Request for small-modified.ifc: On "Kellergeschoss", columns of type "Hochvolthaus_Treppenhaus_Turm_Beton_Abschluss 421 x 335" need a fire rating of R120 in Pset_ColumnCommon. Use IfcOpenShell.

First a look at what the model holds.

```python
import ifcopenshell
import ifcopenshell.util.element

model = ifcopenshell.open("small-modified.ifc")
print(model.schema)
storey = next(s for s in model.by_type("IfcBuildingStorey") if s.Name == "Kellergeschoss")
columns = [e for e in ifcopenshell.util.element.get_decomposition(storey) if e.is_a("IfcColumn")]
seen = {}
for e in columns:
    element_type = ifcopenshell.util.element.get_type(e)
    key = (element_type.Name if element_type != e and element_type else None, ifcopenshell.util.element.get_pset(e, "Pset_ColumnCommon", "FireRating"))
    seen[key] = seen.get(key, 0) + 1
for (name, value), count in sorted(seen.items(), key=str):
    print(count, "x", name, "|", value)
```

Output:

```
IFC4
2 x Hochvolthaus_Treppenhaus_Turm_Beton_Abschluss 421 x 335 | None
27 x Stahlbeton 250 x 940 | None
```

```python
import ifcopenshell
import ifcopenshell.api.pset
import ifcopenshell.util.element

model = ifcopenshell.open("small-modified.ifc")

storey = next(s for s in model.by_type("IfcBuildingStorey") if s.Name == "Kellergeschoss")
columns = [e for e in ifcopenshell.util.element.get_decomposition(storey) if e.is_a("IfcColumn")]

count = 0
for e in columns:
    element_type = ifcopenshell.util.element.get_type(e)
    if element_type in (None, e) or element_type.Name != "Hochvolthaus_Treppenhaus_Turm_Beton_Abschluss 421 x 335":
        continue
    # add_pset returns the element's existing set when there is one.
    pset = ifcopenshell.api.pset.add_pset(model, product=e, name="Pset_ColumnCommon")
    ifcopenshell.api.pset.edit_pset(model, pset=pset, properties={"FireRating": "R120"})
    count += 1

print(count, "columns updated")

model.write("small-modified_edited.ifc")
```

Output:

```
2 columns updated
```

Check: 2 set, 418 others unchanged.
